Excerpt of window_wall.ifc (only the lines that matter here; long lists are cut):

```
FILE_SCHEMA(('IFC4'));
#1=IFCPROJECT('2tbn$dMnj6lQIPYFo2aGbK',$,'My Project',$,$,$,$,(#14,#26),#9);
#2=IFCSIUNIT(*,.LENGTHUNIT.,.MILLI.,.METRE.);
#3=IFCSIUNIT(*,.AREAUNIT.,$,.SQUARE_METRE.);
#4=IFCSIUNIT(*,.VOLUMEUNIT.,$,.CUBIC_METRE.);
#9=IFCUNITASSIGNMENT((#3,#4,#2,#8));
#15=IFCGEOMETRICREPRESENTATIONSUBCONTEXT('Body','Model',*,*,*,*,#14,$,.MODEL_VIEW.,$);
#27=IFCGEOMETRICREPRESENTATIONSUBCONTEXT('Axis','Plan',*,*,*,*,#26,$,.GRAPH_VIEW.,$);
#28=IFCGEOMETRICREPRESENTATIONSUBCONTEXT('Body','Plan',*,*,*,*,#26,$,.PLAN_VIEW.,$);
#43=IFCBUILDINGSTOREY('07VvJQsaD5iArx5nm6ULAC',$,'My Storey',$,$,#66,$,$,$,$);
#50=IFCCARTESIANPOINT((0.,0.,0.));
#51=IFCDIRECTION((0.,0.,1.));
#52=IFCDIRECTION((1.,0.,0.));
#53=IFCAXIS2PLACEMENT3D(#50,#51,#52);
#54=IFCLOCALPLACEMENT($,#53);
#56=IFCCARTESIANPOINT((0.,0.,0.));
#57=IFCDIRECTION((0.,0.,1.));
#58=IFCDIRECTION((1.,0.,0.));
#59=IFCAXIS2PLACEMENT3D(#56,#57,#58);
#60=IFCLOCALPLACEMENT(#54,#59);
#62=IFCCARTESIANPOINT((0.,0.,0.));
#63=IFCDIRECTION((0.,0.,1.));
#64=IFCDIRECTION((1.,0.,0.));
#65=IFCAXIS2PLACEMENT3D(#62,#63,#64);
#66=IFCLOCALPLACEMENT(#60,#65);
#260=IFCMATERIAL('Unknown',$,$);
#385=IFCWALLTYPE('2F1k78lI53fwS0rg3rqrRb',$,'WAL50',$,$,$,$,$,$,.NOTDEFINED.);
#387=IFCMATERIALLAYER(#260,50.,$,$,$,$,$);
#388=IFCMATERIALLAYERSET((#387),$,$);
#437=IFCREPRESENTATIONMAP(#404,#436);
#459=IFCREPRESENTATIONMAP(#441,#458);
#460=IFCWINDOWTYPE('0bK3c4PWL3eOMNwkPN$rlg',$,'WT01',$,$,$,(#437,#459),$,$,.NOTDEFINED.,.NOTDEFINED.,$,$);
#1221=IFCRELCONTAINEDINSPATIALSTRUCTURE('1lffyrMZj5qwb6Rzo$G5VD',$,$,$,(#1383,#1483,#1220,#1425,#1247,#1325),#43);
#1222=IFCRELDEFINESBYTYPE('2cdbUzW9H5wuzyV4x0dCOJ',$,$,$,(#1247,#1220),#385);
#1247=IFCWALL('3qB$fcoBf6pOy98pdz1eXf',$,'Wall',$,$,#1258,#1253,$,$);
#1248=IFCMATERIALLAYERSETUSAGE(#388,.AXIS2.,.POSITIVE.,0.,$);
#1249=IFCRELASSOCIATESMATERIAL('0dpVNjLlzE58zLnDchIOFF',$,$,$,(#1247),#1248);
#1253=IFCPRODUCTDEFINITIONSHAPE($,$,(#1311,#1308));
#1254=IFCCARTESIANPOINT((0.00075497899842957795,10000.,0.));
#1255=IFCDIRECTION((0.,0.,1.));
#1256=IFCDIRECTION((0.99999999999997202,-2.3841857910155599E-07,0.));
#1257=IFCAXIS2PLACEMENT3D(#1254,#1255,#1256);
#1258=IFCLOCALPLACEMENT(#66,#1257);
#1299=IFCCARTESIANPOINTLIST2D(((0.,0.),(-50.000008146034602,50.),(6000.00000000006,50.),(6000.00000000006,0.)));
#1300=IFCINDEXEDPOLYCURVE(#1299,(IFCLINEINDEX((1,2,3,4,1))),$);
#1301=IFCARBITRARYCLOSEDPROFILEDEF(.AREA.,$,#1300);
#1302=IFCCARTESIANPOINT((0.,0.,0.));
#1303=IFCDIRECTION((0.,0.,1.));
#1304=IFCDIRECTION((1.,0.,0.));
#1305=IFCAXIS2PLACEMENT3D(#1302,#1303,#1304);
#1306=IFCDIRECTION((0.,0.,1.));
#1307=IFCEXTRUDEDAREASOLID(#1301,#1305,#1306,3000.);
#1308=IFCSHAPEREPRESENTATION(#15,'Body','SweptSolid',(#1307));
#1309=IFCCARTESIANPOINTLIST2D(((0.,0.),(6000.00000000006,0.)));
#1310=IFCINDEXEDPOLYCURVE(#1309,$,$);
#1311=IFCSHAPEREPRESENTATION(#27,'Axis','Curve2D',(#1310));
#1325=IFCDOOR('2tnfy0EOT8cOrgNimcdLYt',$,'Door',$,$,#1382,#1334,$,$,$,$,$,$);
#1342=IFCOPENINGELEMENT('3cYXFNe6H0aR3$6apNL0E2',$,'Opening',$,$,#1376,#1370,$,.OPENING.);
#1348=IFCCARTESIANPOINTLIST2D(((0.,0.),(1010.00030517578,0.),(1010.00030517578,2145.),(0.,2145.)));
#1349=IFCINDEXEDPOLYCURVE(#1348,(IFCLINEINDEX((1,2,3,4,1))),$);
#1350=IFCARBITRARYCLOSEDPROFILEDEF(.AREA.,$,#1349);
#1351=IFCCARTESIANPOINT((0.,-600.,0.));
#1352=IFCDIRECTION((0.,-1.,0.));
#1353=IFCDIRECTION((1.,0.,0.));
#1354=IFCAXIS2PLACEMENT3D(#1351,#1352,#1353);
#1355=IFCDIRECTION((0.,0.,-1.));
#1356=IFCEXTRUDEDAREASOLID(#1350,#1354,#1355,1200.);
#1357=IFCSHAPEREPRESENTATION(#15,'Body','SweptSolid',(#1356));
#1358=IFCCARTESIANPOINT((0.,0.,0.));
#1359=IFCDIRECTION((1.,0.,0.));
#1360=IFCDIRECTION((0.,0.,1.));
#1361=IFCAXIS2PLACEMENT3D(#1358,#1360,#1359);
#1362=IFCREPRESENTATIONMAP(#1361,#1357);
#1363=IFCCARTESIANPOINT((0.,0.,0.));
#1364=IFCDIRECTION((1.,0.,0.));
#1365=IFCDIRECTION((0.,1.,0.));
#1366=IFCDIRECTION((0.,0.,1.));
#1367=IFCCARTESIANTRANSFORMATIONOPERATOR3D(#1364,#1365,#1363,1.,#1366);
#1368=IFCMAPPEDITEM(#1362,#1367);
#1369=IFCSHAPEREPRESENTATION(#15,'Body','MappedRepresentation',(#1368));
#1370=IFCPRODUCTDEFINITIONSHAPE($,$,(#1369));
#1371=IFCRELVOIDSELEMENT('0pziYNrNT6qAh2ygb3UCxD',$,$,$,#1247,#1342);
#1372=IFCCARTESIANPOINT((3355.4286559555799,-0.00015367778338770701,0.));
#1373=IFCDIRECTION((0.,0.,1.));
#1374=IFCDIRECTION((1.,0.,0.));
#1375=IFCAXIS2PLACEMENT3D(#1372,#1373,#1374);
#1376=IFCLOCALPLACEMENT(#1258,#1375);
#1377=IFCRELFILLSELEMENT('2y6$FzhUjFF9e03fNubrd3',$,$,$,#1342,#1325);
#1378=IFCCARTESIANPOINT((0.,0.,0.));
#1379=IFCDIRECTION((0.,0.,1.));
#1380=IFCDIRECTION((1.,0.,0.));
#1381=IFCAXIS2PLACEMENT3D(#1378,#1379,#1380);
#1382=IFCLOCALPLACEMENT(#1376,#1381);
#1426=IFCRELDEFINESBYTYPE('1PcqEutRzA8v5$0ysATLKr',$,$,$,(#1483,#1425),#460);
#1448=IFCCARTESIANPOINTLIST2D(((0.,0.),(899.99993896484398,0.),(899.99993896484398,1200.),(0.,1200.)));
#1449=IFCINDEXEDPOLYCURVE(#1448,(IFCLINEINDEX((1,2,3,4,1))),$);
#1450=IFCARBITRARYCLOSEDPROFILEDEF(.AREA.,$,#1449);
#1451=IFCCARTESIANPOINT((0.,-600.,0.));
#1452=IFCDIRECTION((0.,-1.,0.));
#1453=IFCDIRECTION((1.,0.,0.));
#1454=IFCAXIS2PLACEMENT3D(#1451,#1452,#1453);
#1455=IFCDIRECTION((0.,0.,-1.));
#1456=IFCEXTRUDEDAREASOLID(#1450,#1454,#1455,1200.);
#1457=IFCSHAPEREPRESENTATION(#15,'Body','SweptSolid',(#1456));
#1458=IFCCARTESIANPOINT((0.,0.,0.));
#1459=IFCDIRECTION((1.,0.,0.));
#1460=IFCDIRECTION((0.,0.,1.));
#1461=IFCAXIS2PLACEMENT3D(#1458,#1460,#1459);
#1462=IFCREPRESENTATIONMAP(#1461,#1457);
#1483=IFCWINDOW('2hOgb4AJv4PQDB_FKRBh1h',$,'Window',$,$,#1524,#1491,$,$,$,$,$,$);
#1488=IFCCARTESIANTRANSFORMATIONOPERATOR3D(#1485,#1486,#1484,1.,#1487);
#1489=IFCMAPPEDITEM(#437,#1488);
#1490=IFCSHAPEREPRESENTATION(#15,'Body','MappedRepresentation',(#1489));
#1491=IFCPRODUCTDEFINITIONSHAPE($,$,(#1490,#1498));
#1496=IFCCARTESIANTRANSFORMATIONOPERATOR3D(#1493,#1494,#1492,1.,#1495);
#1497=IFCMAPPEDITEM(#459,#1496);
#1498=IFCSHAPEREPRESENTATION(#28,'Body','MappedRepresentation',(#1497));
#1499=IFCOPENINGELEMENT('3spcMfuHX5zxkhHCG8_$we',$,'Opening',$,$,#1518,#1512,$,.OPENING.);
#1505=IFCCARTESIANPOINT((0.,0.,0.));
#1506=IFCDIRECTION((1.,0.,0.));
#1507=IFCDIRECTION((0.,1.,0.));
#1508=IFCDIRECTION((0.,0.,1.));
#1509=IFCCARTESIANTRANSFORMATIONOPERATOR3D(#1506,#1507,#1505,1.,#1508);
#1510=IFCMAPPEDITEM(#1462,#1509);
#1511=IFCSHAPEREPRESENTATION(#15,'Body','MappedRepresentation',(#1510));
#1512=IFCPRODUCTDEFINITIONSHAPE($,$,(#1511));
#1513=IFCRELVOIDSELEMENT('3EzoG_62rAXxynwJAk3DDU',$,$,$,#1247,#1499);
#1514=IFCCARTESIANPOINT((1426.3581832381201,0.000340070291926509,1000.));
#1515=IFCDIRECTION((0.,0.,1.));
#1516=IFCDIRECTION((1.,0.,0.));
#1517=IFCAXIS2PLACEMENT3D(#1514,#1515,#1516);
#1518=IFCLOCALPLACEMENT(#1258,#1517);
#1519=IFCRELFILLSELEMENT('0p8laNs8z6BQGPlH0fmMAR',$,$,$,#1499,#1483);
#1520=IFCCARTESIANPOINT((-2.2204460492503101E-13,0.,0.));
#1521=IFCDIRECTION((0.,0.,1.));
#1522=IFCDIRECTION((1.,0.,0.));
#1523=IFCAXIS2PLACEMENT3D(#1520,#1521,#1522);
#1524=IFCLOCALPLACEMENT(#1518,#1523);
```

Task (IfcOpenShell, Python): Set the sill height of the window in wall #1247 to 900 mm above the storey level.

```python
import numpy as np
import ifcopenshell
import ifcopenshell.api.geometry
import ifcopenshell.geom
import ifcopenshell.util.element
import ifcopenshell.util.placement
import ifcopenshell.util.shape
import ifcopenshell.util.unit

model = ifcopenshell.open("window_wall.ifc")
unit_scale = ifcopenshell.util.unit.calculate_unit_scale(model)

window = model.by_guid("2hOgb4AJv4PQDB_FKRBh1h")
opening = window.FillsVoids[0].RelatingOpeningElement
storey = ifcopenshell.util.element.get_container(window, ifc_class="IfcBuildingStorey")
level = ifcopenshell.util.placement.get_local_placement(storey.ObjectPlacement)[2, 3]

# The opening's origin need not be at the sill, so measure its lowest point.
shape = ifcopenshell.geom.create_shape(ifcopenshell.geom.settings(), opening)
bottom = ifcopenshell.util.shape.get_shape_bottom_elevation(shape, shape.geometry) / unit_scale
dz = level + 0.9 / unit_scale - bottom

shift = np.array([0.0, 0.0, dz])
# The window is placed relative to its opening, so it follows when the opening moves.
matrix = ifcopenshell.util.placement.get_local_placement(opening.ObjectPlacement)
matrix[:3, 3] += shift
ifcopenshell.api.geometry.edit_object_placement(
    model, product=opening, matrix=matrix, is_si=False, should_transform_children=True
)

print(f"moved by {dz * unit_scale:+.3f} m")

model.write("window_wall_v2.ifc")
```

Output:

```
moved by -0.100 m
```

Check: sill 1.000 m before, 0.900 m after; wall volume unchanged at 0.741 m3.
